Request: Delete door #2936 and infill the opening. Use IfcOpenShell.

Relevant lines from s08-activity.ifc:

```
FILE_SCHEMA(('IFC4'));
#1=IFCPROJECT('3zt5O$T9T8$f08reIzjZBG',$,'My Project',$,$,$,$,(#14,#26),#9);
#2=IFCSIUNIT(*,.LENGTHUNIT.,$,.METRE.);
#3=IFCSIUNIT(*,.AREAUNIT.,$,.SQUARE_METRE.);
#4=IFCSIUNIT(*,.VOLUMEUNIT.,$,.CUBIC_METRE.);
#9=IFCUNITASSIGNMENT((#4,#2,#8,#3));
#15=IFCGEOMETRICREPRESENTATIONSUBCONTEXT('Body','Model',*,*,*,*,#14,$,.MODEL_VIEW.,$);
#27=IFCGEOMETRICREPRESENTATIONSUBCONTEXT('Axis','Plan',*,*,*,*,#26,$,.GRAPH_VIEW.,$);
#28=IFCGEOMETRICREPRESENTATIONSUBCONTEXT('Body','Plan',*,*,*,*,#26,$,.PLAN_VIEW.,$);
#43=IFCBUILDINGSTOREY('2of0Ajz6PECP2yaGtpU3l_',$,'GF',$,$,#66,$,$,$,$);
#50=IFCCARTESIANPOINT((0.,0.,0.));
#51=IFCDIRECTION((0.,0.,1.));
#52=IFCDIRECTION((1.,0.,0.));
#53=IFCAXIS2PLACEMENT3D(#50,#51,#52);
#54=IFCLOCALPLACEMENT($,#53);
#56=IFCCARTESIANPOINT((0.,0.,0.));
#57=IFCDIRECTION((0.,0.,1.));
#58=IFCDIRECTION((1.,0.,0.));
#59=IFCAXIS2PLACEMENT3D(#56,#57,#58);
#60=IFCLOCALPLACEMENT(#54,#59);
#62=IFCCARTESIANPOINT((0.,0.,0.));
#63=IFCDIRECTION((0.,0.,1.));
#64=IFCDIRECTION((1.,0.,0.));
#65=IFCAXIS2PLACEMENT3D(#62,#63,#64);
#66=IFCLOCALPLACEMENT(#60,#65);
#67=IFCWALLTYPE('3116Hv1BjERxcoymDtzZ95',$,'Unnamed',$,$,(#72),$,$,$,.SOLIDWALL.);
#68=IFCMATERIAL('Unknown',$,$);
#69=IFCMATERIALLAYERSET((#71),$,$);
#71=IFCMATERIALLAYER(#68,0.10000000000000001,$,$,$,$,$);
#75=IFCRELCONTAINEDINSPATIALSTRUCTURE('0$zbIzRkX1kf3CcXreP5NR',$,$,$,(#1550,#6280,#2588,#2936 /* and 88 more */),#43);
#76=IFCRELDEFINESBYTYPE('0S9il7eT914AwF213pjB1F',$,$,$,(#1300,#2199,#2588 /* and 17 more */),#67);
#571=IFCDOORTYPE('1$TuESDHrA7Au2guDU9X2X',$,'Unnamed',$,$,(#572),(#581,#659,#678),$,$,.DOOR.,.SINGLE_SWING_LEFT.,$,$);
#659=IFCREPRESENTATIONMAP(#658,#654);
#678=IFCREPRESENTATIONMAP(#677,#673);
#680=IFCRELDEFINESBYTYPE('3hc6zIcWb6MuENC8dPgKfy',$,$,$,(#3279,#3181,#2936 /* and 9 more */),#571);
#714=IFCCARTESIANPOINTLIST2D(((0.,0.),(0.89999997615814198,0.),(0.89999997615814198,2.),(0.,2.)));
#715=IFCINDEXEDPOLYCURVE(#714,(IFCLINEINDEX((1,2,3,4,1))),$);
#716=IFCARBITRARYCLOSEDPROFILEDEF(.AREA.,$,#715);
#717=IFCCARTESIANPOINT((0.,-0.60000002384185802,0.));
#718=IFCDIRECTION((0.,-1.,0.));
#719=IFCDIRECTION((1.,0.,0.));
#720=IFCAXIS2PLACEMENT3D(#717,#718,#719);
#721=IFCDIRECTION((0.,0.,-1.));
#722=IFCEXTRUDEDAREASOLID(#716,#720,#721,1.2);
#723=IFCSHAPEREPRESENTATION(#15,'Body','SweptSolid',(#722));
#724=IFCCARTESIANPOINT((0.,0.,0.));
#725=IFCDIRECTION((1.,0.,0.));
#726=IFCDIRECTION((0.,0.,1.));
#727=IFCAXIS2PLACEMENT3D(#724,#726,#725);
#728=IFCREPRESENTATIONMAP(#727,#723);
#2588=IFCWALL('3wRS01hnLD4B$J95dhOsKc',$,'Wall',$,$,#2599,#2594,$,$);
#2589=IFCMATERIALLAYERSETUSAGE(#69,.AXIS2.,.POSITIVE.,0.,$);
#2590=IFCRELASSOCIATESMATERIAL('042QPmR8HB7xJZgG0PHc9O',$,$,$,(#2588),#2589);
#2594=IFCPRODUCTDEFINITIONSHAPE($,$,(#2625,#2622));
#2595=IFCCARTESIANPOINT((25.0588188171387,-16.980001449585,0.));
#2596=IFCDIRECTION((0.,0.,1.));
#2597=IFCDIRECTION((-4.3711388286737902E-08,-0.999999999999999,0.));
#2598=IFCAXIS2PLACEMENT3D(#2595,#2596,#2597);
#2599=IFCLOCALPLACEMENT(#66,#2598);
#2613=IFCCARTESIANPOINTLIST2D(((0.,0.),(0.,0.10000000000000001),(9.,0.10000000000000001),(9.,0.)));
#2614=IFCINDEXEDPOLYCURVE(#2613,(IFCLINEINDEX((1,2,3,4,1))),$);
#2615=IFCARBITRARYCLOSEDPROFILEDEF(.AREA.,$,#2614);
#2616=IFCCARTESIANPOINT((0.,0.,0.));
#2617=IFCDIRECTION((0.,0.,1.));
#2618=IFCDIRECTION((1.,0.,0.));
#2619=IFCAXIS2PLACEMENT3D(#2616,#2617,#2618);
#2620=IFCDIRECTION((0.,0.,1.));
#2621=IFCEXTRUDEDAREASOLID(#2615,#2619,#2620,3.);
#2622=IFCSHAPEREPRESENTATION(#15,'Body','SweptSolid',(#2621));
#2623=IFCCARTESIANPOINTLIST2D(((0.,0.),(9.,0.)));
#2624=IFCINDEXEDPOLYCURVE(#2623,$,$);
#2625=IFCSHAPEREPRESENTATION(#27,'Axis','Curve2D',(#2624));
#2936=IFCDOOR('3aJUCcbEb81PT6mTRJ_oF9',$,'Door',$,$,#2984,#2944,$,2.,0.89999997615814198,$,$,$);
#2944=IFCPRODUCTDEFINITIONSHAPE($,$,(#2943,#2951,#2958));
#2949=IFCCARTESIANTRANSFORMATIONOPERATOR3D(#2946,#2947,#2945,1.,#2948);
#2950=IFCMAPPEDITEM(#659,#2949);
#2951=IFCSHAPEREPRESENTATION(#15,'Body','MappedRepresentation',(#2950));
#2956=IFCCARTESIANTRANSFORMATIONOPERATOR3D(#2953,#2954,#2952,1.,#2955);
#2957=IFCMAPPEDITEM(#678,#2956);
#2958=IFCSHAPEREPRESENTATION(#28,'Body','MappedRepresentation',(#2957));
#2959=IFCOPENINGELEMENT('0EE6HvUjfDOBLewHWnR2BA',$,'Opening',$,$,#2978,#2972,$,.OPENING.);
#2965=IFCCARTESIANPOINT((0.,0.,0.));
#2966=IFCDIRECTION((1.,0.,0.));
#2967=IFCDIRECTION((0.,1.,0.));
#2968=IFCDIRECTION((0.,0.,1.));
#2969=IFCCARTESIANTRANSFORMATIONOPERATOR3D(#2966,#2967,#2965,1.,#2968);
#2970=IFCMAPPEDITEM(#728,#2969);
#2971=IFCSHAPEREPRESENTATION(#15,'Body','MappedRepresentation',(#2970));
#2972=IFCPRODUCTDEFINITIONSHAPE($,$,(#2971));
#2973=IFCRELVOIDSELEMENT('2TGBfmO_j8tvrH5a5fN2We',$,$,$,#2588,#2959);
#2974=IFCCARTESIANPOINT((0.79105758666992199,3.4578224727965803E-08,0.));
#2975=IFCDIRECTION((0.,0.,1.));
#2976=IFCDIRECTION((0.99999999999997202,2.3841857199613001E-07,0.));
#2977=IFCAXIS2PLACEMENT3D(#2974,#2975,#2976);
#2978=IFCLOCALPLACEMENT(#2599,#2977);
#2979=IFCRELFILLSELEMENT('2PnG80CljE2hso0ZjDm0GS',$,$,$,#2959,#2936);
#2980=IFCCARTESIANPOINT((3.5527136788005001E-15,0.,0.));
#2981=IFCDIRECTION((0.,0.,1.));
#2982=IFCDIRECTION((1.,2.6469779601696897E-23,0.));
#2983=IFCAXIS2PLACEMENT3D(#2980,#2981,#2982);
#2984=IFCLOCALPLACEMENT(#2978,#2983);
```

```python
import ifcopenshell
import ifcopenshell.api.feature
import ifcopenshell.api.root
import ifcopenshell.geom
import ifcopenshell.util.shape

model = ifcopenshell.open("s08-activity.ifc")
settings = ifcopenshell.geom.settings()


def volume(element):
    """Net volume in cubic metres, openings subtracted."""
    shape = ifcopenshell.geom.create_shape(settings, element)
    return ifcopenshell.util.shape.get_volume(shape.geometry)


door = model.by_guid("3aJUCcbEb81PT6mTRJ_oF9")
opening = door.FillsVoids[0].RelatingOpeningElement
wall = opening.VoidsElements[0].RelatingBuildingElement
before = volume(wall)

ifcopenshell.api.root.remove_product(model, product=door)
ifcopenshell.api.feature.remove_feature(model, feature=opening)

after = volume(wall)

print(f"wall volume {before:.3f} -> {after:.3f} m3")

model.write("s08-activity_rev.ifc")
```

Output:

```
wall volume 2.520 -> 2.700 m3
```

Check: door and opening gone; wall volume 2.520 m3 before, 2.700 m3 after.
